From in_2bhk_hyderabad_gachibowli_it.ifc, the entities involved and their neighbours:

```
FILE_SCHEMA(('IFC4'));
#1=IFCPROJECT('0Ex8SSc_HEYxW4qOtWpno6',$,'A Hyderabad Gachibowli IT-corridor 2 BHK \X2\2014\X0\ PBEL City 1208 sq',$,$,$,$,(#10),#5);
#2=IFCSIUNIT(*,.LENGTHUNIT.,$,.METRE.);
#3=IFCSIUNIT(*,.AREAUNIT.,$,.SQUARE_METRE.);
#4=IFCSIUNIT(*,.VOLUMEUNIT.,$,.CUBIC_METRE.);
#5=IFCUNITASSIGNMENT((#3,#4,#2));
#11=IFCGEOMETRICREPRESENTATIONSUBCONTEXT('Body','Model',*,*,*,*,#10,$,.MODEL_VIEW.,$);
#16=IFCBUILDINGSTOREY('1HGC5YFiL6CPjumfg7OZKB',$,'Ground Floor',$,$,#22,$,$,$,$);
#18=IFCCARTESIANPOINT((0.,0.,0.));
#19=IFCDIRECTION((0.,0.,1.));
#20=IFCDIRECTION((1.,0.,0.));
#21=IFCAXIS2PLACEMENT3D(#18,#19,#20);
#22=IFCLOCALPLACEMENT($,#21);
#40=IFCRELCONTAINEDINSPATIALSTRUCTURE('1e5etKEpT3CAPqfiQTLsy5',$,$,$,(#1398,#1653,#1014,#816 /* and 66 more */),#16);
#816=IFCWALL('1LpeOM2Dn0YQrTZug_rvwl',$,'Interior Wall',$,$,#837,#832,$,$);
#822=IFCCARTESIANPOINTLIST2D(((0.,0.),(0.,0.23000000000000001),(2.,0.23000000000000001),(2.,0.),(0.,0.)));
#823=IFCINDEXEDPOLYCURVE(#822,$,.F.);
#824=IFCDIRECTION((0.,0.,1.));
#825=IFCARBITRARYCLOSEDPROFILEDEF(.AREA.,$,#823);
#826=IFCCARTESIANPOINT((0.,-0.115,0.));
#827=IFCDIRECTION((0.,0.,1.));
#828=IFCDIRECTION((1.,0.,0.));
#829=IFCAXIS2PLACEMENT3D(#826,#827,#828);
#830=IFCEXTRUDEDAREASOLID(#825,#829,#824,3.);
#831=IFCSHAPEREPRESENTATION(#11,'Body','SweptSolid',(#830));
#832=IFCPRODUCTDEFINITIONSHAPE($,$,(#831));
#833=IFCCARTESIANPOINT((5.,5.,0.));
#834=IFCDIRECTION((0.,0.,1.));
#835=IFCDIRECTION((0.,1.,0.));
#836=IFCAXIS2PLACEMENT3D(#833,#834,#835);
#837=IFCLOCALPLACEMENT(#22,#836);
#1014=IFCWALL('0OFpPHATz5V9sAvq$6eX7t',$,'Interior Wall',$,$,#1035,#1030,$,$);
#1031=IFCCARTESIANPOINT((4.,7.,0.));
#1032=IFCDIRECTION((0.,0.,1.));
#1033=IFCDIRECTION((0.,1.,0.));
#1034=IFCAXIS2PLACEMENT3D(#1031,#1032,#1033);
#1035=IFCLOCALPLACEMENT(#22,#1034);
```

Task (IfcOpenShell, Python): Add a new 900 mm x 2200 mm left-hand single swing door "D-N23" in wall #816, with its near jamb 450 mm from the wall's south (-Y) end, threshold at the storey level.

```python
import numpy as np
import ifcopenshell
import ifcopenshell.api.feature
import ifcopenshell.api.geometry
import ifcopenshell.api.root
import ifcopenshell.api.spatial
import ifcopenshell.geom
import ifcopenshell.util.element
import ifcopenshell.util.placement
import ifcopenshell.util.representation
import ifcopenshell.util.shape
import ifcopenshell.util.unit

model = ifcopenshell.open("in_2bhk_hyderabad_gachibowli_it.ifc")
unit_scale = ifcopenshell.util.unit.calculate_unit_scale(model)
settings = ifcopenshell.geom.settings()


def volume(element):
    """Net volume in cubic metres, openings subtracted."""
    shape = ifcopenshell.geom.create_shape(settings, element)
    return ifcopenshell.util.shape.get_volume(shape.geometry)


wall = model.by_guid("1LpeOM2Dn0YQrTZug_rvwl")
storey = ifcopenshell.util.element.get_container(wall, ifc_class="IfcBuildingStorey")
context = ifcopenshell.util.representation.get_context(model, "Model", "Body", "MODEL_VIEW")
before = volume(wall)

width, height, from_end, sill = 0.9, 2.2, 0.45, 0.0  # metres

# The wall runs along its own X axis, and the end named is its -X end.
wall_shape = ifcopenshell.geom.create_shape(settings, wall)
x, y, z = ifcopenshell.util.shape.get_vertices(wall_shape.geometry).T
start = x.min() + from_end
face, thickness = float(y.min()), float(y.max() - y.min())
wall_matrix = ifcopenshell.util.placement.get_local_placement(wall.ObjectPlacement)
level = ifcopenshell.util.placement.get_local_placement(storey.ObjectPlacement)[2, 3]


def in_wall(x, y):
    """Placement at x, y metres in the wall's axes, at sill height."""
    matrix = wall_matrix.copy()
    matrix[:, 3] = wall_matrix @ np.array([x / unit_scale, y / unit_scale, 0.0, 1.0])
    matrix[2, 3] = level + sill / unit_scale
    return matrix


# Opening: a box that overshoots both wall faces by 50 mm.
opening = ifcopenshell.api.root.create_entity(model, ifc_class="IfcOpeningElement", predefined_type="OPENING")
box = ifcopenshell.api.geometry.add_wall_representation(
    model, context=context, length=width, height=height, thickness=thickness + 0.1
)
ifcopenshell.api.geometry.assign_representation(model, product=opening, representation=box)
ifcopenshell.api.geometry.edit_object_placement(model, product=opening, matrix=in_wall(start, face - 0.05), is_si=False)
ifcopenshell.api.feature.add_feature(model, feature=opening, element=wall)

door = ifcopenshell.api.root.create_entity(model, ifc_class="IfcDoor", name="D-N23", predefined_type="DOOR")
door.OverallWidth, door.OverallHeight = width / unit_scale, height / unit_scale
door.OperationType = "SINGLE_SWING_LEFT"
body = ifcopenshell.api.geometry.add_door_representation(
    model,
    context=context,
    overall_width=door.OverallWidth,
    overall_height=door.OverallHeight,
    operation_type="SINGLE_SWING_LEFT",
    lining_properties={"LiningDepth": thickness / unit_scale, "ThresholdDepth": thickness / unit_scale},
)
ifcopenshell.api.geometry.assign_representation(model, product=door, representation=body)
ifcopenshell.api.spatial.assign_container(model, products=[door], relating_structure=storey)
ifcopenshell.api.feature.add_filling(model, opening=opening, element=door)

# The lining spans the wall, so the door starts at the wall face.
ifcopenshell.api.geometry.edit_object_placement(model, product=door, matrix=in_wall(start, face), is_si=False)

after = volume(wall)

print(f"wall volume {before:.3f} -> {after:.3f} m3")

model.write("in_2bhk_hyderabad_gachibowli_it_v2.ifc")
```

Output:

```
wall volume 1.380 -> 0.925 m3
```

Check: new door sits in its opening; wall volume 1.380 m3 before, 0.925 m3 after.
